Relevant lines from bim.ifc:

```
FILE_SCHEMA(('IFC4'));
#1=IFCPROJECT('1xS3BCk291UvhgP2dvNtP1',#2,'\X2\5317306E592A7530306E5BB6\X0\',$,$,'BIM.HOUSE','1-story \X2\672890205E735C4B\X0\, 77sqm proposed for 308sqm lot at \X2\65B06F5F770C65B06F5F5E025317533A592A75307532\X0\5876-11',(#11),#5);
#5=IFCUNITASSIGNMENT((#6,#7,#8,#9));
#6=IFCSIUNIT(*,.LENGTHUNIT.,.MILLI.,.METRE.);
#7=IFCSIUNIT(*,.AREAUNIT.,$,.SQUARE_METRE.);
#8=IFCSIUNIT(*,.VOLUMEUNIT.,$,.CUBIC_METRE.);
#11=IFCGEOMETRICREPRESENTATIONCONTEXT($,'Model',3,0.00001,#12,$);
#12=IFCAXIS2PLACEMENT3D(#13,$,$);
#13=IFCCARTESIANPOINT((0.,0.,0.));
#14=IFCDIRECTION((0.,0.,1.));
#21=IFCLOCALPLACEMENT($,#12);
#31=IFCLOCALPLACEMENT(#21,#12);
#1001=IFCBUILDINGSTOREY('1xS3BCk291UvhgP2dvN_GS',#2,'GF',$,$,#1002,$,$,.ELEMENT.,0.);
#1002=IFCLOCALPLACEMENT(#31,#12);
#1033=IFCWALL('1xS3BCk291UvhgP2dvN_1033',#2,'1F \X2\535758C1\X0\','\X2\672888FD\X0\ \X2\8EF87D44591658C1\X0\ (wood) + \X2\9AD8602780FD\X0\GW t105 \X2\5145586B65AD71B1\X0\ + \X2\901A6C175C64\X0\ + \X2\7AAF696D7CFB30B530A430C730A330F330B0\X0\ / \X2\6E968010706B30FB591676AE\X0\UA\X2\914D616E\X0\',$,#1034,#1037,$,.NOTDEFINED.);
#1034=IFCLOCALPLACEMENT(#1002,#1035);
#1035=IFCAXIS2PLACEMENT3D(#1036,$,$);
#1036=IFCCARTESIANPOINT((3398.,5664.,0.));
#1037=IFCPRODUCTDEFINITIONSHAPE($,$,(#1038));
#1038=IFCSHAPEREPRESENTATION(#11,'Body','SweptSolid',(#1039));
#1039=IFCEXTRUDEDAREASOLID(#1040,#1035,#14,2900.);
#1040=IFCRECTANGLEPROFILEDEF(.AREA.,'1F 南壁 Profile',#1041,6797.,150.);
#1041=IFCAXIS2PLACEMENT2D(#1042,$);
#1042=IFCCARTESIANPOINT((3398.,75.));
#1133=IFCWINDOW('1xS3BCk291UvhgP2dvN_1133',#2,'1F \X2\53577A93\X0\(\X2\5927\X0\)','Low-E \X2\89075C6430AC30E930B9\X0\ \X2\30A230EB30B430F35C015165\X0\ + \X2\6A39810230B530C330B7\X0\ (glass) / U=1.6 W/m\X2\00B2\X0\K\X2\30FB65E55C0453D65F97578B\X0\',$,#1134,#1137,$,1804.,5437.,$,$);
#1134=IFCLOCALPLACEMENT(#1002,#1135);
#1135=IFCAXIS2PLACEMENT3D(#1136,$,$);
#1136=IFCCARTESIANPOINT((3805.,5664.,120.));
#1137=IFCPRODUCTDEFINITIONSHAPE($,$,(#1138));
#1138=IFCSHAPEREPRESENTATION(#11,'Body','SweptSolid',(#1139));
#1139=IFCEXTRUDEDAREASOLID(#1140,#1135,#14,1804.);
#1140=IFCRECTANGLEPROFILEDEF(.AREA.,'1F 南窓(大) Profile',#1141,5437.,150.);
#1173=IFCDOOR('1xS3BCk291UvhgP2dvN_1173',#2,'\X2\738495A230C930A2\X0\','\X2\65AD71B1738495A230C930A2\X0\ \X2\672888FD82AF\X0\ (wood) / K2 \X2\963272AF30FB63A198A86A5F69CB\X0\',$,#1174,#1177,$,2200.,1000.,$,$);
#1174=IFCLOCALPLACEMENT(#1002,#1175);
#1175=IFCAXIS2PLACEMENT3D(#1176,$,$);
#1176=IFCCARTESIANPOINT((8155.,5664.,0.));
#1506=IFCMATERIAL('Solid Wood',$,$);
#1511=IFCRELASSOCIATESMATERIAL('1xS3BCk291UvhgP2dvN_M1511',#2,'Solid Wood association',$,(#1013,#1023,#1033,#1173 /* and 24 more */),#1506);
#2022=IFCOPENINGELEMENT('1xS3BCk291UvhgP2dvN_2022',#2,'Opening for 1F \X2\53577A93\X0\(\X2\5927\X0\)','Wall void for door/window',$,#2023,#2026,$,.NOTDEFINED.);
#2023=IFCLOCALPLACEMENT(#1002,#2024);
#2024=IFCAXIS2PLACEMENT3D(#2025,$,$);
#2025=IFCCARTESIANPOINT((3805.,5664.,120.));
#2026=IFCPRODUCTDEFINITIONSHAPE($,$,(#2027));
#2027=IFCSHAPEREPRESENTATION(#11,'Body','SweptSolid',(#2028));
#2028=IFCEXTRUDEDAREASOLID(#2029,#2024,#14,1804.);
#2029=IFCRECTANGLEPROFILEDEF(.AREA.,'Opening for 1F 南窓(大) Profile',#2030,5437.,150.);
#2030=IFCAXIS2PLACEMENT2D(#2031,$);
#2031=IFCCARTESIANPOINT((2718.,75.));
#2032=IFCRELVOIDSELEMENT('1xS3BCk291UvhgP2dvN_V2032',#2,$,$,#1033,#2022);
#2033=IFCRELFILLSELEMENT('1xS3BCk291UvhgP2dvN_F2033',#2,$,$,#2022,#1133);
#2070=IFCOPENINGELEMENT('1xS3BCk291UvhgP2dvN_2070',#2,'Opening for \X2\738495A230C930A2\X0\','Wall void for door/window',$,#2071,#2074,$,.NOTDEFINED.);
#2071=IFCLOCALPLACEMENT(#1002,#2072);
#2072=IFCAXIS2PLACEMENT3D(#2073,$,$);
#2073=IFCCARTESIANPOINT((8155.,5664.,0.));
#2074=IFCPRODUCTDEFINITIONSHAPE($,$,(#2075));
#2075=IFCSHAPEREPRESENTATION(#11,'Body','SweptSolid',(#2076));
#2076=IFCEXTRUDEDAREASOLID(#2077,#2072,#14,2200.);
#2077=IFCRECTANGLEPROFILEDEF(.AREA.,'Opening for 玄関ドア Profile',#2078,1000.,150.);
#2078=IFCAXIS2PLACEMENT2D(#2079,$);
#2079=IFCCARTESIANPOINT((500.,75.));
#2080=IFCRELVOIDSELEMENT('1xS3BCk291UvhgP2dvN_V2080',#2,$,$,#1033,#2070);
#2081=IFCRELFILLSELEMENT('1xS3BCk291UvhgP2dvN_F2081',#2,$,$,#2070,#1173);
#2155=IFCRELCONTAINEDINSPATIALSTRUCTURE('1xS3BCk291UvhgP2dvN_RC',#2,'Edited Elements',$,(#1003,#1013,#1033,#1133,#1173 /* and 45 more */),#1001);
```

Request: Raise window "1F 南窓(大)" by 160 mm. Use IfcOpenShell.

```python
import numpy as np
import ifcopenshell
import ifcopenshell.api.geometry
import ifcopenshell.util.placement
import ifcopenshell.util.unit

model = ifcopenshell.open("bim.ifc")
unit_scale = ifcopenshell.util.unit.calculate_unit_scale(model)

window = model.by_guid("1xS3BCk291UvhgP2dvN_1133")
opening = window.FillsVoids[0].RelatingOpeningElement
dz = 0.16 / unit_scale

shift = np.array([0.0, 0.0, dz])
# The window is not placed relative to its opening, so move both.
for product in (opening, window):
    matrix = ifcopenshell.util.placement.get_local_placement(product.ObjectPlacement)
    matrix[:3, 3] += shift
    ifcopenshell.api.geometry.edit_object_placement(model, product=product, matrix=matrix, is_si=False)

print(f"moved by {dz * unit_scale:+.3f} m")

model.write("bim_updated.ifc")
```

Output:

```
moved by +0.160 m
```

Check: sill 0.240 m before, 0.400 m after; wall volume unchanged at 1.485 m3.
